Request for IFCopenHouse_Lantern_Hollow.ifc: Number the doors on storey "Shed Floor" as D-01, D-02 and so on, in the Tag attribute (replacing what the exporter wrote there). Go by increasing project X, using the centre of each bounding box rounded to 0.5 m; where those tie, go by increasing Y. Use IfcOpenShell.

First a look at what the model holds.

```python
import ifcopenshell
import ifcopenshell.util.element
import ifcopenshell.util.placement

model = ifcopenshell.open("IFCopenHouse_Lantern_Hollow.ifc")
print(model.schema)
storey = next(s for s in model.by_type("IfcBuildingStorey") if s.Name == "Shed Floor")
doors = [e for e in ifcopenshell.util.element.get_decomposition(storey) if e.is_a("IfcDoor")]
for e in sorted(doors, key=lambda e: e.id()):
    origin = ifcopenshell.util.placement.get_local_placement(e.ObjectPlacement)[:3, 3]
    print(e.id(), e.Tag, e.Name, origin.round(2) + 0.0, sep=" | ")
```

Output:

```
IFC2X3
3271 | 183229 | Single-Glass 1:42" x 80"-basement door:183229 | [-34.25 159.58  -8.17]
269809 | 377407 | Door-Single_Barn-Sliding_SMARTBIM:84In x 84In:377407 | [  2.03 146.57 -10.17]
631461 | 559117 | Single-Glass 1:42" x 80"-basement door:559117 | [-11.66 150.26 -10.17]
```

```python
import ifcopenshell
import ifcopenshell.geom
import ifcopenshell.util.element
import ifcopenshell.util.shape

model = ifcopenshell.open("IFCopenHouse_Lantern_Hollow.ifc")
settings = ifcopenshell.geom.settings()
settings.set("use-world-coords", True)


def centre(element):
    shape = ifcopenshell.geom.create_shape(settings, element)
    return ifcopenshell.util.shape.get_bbox_centroid(shape.geometry)


storey = next(s for s in model.by_type("IfcBuildingStorey") if s.Name == "Shed Floor")
doors = [e for e in ifcopenshell.util.element.get_decomposition(storey) if e.is_a("IfcDoor")]

# Insertion points can sit at a corner or the storey origin, so sort by the geometry (in metres).
centres = {e: centre(e) for e in doors}
doors.sort(key=lambda e: (round(centres[e][0] / 0.5), centres[e][1]))

for i, e in enumerate(doors, start=1):
    number = f"D-{i:02d}"
    e.Tag = number
    print(e.id(), number)

model.write("IFCopenHouse_Lantern_Hollow-out.ifc")
```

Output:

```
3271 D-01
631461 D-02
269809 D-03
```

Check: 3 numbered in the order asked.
